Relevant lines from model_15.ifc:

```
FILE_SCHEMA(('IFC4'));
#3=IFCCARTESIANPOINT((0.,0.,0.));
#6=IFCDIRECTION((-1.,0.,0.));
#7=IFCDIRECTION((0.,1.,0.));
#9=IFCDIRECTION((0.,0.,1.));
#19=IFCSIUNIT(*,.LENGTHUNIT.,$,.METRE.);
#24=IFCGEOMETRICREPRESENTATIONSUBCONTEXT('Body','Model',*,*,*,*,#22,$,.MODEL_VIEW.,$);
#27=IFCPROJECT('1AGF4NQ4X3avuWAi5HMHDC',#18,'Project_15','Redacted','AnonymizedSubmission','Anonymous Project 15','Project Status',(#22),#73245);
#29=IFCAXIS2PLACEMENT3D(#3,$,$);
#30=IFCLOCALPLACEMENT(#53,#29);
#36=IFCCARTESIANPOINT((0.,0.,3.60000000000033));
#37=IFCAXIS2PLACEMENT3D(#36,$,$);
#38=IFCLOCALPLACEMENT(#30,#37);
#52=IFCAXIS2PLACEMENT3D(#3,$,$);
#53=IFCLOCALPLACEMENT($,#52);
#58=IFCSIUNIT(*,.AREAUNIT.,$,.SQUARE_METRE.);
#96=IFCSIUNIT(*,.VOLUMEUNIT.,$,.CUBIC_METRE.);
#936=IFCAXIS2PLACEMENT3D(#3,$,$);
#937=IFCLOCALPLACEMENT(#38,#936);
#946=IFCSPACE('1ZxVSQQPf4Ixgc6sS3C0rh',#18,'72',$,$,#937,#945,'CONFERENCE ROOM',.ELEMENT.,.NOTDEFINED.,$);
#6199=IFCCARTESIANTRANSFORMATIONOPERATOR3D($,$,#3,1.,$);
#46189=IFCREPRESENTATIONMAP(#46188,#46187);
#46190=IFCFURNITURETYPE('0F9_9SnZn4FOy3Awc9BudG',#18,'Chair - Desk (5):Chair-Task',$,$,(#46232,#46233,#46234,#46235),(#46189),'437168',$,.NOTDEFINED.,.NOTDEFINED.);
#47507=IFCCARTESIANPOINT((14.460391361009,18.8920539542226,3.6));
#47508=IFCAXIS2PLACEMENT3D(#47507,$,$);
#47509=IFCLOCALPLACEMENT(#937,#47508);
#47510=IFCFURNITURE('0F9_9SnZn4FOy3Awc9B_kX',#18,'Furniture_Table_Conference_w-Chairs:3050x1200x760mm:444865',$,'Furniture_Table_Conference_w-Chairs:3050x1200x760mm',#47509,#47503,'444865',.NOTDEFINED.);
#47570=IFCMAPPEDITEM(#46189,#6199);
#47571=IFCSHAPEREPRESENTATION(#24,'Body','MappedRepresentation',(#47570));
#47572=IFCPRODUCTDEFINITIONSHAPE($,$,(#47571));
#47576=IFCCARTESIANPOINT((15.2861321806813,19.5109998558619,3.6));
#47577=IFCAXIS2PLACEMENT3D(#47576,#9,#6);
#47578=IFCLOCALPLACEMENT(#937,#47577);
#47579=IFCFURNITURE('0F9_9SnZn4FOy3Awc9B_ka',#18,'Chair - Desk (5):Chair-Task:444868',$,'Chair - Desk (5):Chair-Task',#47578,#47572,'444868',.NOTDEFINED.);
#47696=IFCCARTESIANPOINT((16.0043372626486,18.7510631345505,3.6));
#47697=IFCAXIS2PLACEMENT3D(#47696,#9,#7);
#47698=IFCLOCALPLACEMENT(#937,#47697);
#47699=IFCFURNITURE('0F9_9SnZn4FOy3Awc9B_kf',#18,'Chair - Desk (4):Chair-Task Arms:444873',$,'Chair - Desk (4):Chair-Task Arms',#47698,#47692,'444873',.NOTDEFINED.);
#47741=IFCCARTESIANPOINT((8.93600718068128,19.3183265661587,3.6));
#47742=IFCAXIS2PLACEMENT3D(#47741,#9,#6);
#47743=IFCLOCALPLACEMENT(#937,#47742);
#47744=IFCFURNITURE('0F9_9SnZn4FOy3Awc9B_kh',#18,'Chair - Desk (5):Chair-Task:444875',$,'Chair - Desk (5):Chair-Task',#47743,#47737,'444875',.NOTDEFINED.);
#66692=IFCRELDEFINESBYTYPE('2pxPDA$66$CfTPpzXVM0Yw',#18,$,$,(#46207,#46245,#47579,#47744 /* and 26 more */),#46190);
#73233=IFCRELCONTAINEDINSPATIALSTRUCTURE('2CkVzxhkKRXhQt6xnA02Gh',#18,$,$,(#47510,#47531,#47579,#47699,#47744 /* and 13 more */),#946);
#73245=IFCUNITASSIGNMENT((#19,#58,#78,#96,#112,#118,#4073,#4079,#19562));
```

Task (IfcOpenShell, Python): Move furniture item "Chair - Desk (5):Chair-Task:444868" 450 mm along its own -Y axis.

```python
import ifcopenshell
import ifcopenshell.api.geometry
import ifcopenshell.util.placement
import ifcopenshell.util.unit

model = ifcopenshell.open("model_15.ifc")
unit_scale = ifcopenshell.util.unit.calculate_unit_scale(model)

item = model.by_guid("0F9_9SnZn4FOy3Awc9B_ka")
matrix = ifcopenshell.util.placement.get_local_placement(item.ObjectPlacement)
matrix[:3, 3] -= matrix[:3, 1] * 0.45 / unit_scale
ifcopenshell.api.geometry.edit_object_placement(model, product=item, matrix=matrix, is_si=False)

print(ifcopenshell.util.placement.get_local_placement(item.ObjectPlacement).round(3) + 0.0)

model.write("model_15_updated.ifc")
```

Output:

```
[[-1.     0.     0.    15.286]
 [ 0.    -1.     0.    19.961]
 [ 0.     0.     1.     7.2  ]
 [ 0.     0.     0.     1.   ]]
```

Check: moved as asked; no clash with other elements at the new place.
